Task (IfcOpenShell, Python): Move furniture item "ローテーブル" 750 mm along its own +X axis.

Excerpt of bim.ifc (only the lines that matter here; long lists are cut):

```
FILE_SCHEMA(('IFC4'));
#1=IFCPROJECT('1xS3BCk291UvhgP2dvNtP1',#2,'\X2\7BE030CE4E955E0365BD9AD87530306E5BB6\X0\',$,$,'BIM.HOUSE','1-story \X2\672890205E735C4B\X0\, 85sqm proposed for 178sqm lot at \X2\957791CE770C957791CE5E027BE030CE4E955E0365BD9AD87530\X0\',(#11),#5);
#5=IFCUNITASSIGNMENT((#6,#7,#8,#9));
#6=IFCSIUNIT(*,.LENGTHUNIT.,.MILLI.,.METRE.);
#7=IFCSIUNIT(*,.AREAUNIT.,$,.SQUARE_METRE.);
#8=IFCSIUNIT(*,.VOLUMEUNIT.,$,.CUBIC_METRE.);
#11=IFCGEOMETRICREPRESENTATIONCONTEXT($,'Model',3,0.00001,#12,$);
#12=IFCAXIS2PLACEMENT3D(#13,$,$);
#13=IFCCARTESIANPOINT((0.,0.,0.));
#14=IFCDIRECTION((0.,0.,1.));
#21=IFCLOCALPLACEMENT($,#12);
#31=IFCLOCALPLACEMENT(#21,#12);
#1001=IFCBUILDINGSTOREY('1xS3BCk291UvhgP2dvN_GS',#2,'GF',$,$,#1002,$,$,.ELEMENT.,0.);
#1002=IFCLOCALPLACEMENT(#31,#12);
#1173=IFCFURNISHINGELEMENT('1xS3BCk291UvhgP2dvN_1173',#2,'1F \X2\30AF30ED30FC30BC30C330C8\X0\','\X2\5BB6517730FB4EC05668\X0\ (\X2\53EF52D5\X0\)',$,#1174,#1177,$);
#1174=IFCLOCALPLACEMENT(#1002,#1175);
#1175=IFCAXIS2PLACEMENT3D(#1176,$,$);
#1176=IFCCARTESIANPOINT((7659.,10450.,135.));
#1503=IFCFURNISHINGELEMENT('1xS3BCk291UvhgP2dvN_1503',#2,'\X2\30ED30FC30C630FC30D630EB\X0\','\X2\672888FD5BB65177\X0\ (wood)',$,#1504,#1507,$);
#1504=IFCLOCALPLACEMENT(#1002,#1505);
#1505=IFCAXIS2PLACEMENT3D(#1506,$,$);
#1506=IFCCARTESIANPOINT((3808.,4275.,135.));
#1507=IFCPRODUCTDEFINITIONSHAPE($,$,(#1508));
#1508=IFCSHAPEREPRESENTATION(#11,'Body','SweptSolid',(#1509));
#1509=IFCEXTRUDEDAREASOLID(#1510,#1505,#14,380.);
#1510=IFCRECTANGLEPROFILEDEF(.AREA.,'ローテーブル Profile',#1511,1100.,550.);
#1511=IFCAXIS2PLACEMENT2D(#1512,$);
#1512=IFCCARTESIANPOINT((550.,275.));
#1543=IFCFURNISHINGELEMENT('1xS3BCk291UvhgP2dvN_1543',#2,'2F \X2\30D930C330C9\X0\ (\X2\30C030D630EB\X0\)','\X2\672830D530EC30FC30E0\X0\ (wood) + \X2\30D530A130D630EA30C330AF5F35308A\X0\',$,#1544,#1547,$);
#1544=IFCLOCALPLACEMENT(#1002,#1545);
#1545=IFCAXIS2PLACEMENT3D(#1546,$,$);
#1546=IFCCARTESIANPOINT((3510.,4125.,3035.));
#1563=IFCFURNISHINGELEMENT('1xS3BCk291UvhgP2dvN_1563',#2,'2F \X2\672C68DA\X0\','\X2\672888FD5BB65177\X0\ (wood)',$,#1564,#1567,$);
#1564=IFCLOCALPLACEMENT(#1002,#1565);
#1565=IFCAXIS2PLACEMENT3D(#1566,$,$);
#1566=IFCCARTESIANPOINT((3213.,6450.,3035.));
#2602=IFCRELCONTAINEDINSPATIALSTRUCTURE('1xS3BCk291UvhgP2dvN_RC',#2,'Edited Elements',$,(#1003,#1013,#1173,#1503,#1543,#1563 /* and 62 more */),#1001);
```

```python
import ifcopenshell
import ifcopenshell.api.geometry
import ifcopenshell.util.placement
import ifcopenshell.util.unit

model = ifcopenshell.open("bim.ifc")
unit_scale = ifcopenshell.util.unit.calculate_unit_scale(model)

item = model.by_guid("1xS3BCk291UvhgP2dvN_1503")
matrix = ifcopenshell.util.placement.get_local_placement(item.ObjectPlacement)
matrix[:3, 3] += matrix[:3, 0] * 0.75 / unit_scale
ifcopenshell.api.geometry.edit_object_placement(model, product=item, matrix=matrix, is_si=False)

print(ifcopenshell.util.placement.get_local_placement(item.ObjectPlacement).round(3) + 0.0)

model.write("bim_updated.ifc")
```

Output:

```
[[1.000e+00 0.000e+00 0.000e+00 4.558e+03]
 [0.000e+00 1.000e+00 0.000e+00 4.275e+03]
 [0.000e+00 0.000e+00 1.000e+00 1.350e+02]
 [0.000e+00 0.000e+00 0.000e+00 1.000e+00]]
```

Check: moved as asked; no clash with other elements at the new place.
